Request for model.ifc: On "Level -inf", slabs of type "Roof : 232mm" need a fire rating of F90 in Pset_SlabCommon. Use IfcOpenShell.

First a look at what the model holds.

```python
import ifcopenshell
import ifcopenshell.util.element

model = ifcopenshell.open("model.ifc")
print(model.schema)
storey = next(s for s in model.by_type("IfcBuildingStorey") if s.Name == "Level -inf")
slabs = [e for e in ifcopenshell.util.element.get_decomposition(storey) if e.is_a("IfcSlab")]
seen = {}
for e in slabs:
    element_type = ifcopenshell.util.element.get_type(e)
    key = (element_type.Name if element_type != e and element_type else None, ifcopenshell.util.element.get_pset(e, "Pset_SlabCommon", "FireRating"))
    seen[key] = seen.get(key, 0) + 1
for (name, value), count in sorted(seen.items(), key=str):
    print(count, "x", name, "|", value)
```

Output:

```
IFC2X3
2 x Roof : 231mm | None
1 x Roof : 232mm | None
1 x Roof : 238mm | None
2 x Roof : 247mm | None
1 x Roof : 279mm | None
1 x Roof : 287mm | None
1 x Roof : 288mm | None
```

```python
import ifcopenshell
import ifcopenshell.api.pset
import ifcopenshell.util.element

model = ifcopenshell.open("model.ifc")

storey = next(s for s in model.by_type("IfcBuildingStorey") if s.Name == "Level -inf")
slabs = [e for e in ifcopenshell.util.element.get_decomposition(storey) if e.is_a("IfcSlab")]

count = 0
for e in slabs:
    element_type = ifcopenshell.util.element.get_type(e)
    if element_type in (None, e) or element_type.Name != "Roof : 232mm":
        continue
    # add_pset returns the element's existing set when there is one.
    pset = ifcopenshell.api.pset.add_pset(model, product=e, name="Pset_SlabCommon")
    ifcopenshell.api.pset.edit_pset(model, pset=pset, properties={"FireRating": "F90"})
    count += 1

print(count, "slabs updated")

model.write("model_edited.ifc")
```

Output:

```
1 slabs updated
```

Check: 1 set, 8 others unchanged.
